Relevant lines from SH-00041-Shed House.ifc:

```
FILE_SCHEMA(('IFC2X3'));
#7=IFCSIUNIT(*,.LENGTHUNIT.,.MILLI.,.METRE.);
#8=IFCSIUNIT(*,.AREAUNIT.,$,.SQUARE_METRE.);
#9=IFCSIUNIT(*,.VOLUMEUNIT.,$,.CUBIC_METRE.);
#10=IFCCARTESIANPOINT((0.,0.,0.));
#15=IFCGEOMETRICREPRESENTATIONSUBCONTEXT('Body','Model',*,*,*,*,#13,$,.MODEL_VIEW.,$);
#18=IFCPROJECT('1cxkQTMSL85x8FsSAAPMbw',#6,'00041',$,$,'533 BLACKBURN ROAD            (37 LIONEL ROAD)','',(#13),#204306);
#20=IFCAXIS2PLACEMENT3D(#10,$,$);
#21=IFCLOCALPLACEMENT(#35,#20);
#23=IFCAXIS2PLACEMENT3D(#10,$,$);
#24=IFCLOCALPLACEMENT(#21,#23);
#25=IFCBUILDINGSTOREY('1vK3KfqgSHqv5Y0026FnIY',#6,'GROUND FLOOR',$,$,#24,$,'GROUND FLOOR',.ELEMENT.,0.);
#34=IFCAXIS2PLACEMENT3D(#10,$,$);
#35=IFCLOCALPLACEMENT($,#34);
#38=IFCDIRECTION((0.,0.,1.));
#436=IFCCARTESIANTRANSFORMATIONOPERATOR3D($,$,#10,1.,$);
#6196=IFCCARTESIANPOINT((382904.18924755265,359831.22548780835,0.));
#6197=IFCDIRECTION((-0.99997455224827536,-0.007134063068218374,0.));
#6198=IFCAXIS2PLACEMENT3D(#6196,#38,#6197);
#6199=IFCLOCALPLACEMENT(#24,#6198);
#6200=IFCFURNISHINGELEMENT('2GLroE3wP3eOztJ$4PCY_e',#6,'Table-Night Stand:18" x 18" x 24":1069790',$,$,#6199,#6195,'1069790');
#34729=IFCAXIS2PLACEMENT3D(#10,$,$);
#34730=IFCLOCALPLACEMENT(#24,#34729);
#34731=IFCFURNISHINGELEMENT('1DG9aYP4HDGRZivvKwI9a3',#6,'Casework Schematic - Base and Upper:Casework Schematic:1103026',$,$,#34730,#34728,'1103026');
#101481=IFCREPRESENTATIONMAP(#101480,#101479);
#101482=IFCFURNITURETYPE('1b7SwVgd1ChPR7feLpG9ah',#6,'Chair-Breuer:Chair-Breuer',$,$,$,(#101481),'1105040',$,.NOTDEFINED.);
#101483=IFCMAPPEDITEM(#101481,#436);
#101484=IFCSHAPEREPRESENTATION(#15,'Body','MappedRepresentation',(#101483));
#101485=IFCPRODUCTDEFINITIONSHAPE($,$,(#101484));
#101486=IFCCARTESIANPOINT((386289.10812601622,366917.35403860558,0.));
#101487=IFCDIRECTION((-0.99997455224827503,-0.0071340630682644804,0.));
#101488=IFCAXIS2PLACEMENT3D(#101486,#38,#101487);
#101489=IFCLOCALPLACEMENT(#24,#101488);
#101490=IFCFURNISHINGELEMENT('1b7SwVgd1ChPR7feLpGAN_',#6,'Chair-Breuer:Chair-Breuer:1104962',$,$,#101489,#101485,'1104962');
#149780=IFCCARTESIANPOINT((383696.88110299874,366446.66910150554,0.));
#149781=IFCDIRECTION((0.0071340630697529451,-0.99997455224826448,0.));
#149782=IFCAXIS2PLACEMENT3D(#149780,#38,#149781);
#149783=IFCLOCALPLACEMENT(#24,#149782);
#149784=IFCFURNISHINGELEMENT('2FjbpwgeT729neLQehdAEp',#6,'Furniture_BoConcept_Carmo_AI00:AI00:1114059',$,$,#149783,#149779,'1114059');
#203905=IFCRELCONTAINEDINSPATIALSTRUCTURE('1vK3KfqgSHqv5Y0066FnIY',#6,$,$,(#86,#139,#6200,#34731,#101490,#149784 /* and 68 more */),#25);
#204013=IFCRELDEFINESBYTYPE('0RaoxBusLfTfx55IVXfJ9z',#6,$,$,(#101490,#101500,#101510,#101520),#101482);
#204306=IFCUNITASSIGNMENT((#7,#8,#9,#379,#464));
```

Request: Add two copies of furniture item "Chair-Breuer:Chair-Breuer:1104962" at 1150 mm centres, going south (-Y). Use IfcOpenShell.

```python
import numpy as np
import ifcopenshell
import ifcopenshell.api.geometry
import ifcopenshell.api.root
import ifcopenshell.util.element
import ifcopenshell.util.placement

model = ifcopenshell.open("SH-00041-Shed House.ifc")


def reuse_history(source, copy):
    """copy_class also copies each property set's owner history, people and application; keep the originals."""
    for rel in copy.IsDefinedBy:
        if rel.is_a("IfcRelDefinesByProperties") and (history := rel.RelatingPropertyDefinition.OwnerHistory):
            rel.RelatingPropertyDefinition.OwnerHistory = source.OwnerHistory
            ifcopenshell.util.element.remove_deep2(model, history)


source = model.by_guid("1b7SwVgd1ChPR7feLpGAN_")
base = ifcopenshell.util.placement.get_local_placement(source.ObjectPlacement)
step = np.array([0.0, -1.0, 0.0]) * 1150.0

for i in range(1, 3):
    copy = ifcopenshell.api.root.copy_class(model, product=source)
    copy.Representation = ifcopenshell.util.element.copy_deep(
        model, source.Representation, exclude=["IfcGeometricRepresentationContext", "IfcRepresentationMap"]
    )
    copy.Name = "Chair-Breuer:Chair-Breuer"
    copy.Tag = None
    reuse_history(source, copy)
    matrix = base.copy()
    matrix[:3, 3] += i * step
    print("added at", matrix[:3, 3].round(3) + 0.0)
    ifcopenshell.api.geometry.edit_object_placement(model, product=copy, matrix=matrix, is_si=False)

model.write("SH-00041-Shed House-out.ifc")
```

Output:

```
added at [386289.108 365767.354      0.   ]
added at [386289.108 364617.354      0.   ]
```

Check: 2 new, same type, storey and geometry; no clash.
